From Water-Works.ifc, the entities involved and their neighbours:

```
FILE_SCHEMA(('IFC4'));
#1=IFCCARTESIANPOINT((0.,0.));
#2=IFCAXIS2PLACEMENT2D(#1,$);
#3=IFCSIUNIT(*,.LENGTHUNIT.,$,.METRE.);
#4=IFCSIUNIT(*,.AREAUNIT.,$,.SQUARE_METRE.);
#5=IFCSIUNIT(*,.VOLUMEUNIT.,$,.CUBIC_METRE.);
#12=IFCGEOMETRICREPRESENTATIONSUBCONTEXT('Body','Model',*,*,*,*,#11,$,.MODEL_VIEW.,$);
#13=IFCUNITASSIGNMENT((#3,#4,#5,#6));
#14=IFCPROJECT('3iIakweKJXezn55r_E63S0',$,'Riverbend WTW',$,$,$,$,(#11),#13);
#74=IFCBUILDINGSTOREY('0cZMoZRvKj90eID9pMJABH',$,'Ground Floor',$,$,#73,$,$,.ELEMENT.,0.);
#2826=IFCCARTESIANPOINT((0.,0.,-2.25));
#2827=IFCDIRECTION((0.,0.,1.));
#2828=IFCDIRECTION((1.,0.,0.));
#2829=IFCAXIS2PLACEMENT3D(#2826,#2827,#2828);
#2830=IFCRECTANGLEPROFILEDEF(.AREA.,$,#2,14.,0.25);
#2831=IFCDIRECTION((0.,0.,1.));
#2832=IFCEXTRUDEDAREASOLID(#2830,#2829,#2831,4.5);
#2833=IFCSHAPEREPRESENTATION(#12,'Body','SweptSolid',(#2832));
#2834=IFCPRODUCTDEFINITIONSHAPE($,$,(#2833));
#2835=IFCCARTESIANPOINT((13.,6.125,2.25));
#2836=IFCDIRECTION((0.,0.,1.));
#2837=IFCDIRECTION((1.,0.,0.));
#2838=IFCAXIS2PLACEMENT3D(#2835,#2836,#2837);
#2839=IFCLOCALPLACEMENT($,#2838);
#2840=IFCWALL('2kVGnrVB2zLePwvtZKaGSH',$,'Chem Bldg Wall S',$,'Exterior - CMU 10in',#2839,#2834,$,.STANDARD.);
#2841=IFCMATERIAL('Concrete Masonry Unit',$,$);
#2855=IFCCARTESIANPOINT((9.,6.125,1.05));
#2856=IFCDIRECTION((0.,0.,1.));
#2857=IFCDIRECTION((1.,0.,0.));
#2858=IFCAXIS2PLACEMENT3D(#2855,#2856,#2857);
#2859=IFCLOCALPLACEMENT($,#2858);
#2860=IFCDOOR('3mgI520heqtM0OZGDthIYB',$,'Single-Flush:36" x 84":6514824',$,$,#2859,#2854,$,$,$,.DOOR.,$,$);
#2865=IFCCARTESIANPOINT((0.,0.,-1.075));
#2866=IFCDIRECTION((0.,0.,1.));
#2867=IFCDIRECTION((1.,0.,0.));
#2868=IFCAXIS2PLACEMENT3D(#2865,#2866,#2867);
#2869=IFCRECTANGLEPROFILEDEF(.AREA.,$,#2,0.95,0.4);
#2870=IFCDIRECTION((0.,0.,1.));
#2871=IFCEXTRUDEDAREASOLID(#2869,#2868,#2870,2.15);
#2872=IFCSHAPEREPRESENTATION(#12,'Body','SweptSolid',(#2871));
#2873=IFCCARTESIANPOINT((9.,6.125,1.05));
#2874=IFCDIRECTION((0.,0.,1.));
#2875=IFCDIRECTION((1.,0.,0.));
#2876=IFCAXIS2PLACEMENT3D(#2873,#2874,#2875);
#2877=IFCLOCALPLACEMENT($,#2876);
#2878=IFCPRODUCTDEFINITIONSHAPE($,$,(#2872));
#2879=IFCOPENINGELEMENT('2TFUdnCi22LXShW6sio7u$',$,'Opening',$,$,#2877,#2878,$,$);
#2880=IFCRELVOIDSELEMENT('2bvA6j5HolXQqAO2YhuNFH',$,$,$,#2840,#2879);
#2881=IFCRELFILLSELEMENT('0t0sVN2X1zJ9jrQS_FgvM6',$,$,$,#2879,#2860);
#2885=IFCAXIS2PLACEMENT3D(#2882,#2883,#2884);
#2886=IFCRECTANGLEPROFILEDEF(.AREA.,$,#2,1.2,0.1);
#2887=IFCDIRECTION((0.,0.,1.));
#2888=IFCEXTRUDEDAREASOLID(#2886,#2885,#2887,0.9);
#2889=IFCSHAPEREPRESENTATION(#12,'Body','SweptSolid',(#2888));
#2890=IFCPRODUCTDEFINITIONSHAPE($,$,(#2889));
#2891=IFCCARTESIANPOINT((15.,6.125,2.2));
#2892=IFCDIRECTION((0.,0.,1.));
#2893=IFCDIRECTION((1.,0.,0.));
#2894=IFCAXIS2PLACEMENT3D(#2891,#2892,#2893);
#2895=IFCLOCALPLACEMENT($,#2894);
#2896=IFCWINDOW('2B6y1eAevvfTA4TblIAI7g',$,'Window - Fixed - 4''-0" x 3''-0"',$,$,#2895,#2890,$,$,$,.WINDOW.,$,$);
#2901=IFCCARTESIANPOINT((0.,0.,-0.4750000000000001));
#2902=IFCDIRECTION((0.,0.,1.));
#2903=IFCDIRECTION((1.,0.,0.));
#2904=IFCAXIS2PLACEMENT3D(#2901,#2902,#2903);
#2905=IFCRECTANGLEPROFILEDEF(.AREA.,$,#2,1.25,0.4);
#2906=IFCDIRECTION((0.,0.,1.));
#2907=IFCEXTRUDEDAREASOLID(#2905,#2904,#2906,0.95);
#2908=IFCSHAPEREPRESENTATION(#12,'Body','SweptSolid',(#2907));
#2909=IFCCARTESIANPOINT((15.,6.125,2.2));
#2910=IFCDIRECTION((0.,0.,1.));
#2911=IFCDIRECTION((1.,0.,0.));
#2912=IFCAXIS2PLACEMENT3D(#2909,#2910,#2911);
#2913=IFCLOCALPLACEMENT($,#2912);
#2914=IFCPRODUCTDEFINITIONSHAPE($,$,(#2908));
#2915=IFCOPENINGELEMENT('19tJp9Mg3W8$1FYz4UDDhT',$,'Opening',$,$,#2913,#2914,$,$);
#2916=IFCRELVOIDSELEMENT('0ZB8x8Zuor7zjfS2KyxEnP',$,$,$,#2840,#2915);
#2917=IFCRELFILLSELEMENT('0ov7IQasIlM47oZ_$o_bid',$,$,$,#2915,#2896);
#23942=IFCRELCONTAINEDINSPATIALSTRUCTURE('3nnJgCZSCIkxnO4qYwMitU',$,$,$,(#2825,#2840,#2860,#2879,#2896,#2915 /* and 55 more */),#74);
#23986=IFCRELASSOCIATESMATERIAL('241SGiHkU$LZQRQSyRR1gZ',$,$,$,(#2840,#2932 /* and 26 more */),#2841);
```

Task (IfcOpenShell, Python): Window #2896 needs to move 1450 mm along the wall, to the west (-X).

```python
import ifcopenshell
import ifcopenshell.api.geometry
import ifcopenshell.util.placement
import ifcopenshell.util.unit

model = ifcopenshell.open("Water-Works.ifc")
unit_scale = ifcopenshell.util.unit.calculate_unit_scale(model)

window = model.by_guid("2B6y1eAevvfTA4TblIAI7g")
opening = window.FillsVoids[0].RelatingOpeningElement
wall = opening.VoidsElements[0].RelatingBuildingElement

wall_matrix = ifcopenshell.util.placement.get_local_placement(wall.ObjectPlacement)
shift = wall_matrix[:3, 0] * -1.45 / unit_scale
before = ifcopenshell.util.placement.get_local_placement(window.ObjectPlacement)[:3, 3].copy()

# The window is not placed relative to its opening, so move both.
for product in (opening, window):
    matrix = ifcopenshell.util.placement.get_local_placement(product.ObjectPlacement)
    matrix[:3, 3] += shift
    ifcopenshell.api.geometry.edit_object_placement(model, product=product, matrix=matrix, is_si=False)

after = ifcopenshell.util.placement.get_local_placement(window.ObjectPlacement)[:3, 3]
print("window moved by", (after - before).round(3) + 0.0)

model.write("Water-Works_v2.ifc")
```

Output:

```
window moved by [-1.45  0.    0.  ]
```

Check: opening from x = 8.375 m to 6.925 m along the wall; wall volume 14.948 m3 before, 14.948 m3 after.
